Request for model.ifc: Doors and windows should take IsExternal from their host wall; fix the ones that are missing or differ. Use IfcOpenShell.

First a look at what the model holds.

```python
import ifcopenshell
import ifcopenshell.util.element

model = ifcopenshell.open("model.ifc")
print(model.schema)
seen = {}
for e in model.by_type("IfcDoor") + model.by_type("IfcWindow"):
    if not e.FillsVoids:
        continue
    host = e.FillsVoids[0].RelatingOpeningElement.VoidsElements[0].RelatingBuildingElement
    own = ifcopenshell.util.element.get_pset(e, f"Pset_{e.is_a()[3:].removesuffix('StandardCase')}Common", "IsExternal")
    wall = ifcopenshell.util.element.get_pset(host, "Pset_WallCommon", "IsExternal")
    seen[e.is_a(), own, wall] = seen.get((e.is_a(), own, wall), 0) + 1
for (cls, own, wall), count in sorted(seen.items(), key=str):
    print(count, cls, "IsExternal:", own, "| host wall:", wall)
```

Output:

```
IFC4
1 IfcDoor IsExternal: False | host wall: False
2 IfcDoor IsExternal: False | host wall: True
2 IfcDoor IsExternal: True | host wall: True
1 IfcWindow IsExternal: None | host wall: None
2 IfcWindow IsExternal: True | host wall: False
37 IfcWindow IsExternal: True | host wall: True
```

```python
import ifcopenshell
import ifcopenshell.api.pset
import ifcopenshell.util.element

model = ifcopenshell.open("model.ifc")

count = 0
for ifc_class, pset_name in (("IfcDoor", "Pset_DoorCommon"), ("IfcWindow", "Pset_WindowCommon")):
    for e in model.by_type(ifc_class):
        if not e.FillsVoids:
            continue
        host = e.FillsVoids[0].RelatingOpeningElement.VoidsElements[0].RelatingBuildingElement
        external = ifcopenshell.util.element.get_pset(host, "Pset_WallCommon", "IsExternal")
        if external is None or ifcopenshell.util.element.get_pset(e, pset_name, "IsExternal") == external:
            continue
        pset = ifcopenshell.api.pset.add_pset(model, product=e, name=pset_name)
        ifcopenshell.api.pset.edit_pset(model, pset=pset, properties={"IsExternal": external})
        count += 1

print(count, "updated")

model.write("model_updated.ifc")
```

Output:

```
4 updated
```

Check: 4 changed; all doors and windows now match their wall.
